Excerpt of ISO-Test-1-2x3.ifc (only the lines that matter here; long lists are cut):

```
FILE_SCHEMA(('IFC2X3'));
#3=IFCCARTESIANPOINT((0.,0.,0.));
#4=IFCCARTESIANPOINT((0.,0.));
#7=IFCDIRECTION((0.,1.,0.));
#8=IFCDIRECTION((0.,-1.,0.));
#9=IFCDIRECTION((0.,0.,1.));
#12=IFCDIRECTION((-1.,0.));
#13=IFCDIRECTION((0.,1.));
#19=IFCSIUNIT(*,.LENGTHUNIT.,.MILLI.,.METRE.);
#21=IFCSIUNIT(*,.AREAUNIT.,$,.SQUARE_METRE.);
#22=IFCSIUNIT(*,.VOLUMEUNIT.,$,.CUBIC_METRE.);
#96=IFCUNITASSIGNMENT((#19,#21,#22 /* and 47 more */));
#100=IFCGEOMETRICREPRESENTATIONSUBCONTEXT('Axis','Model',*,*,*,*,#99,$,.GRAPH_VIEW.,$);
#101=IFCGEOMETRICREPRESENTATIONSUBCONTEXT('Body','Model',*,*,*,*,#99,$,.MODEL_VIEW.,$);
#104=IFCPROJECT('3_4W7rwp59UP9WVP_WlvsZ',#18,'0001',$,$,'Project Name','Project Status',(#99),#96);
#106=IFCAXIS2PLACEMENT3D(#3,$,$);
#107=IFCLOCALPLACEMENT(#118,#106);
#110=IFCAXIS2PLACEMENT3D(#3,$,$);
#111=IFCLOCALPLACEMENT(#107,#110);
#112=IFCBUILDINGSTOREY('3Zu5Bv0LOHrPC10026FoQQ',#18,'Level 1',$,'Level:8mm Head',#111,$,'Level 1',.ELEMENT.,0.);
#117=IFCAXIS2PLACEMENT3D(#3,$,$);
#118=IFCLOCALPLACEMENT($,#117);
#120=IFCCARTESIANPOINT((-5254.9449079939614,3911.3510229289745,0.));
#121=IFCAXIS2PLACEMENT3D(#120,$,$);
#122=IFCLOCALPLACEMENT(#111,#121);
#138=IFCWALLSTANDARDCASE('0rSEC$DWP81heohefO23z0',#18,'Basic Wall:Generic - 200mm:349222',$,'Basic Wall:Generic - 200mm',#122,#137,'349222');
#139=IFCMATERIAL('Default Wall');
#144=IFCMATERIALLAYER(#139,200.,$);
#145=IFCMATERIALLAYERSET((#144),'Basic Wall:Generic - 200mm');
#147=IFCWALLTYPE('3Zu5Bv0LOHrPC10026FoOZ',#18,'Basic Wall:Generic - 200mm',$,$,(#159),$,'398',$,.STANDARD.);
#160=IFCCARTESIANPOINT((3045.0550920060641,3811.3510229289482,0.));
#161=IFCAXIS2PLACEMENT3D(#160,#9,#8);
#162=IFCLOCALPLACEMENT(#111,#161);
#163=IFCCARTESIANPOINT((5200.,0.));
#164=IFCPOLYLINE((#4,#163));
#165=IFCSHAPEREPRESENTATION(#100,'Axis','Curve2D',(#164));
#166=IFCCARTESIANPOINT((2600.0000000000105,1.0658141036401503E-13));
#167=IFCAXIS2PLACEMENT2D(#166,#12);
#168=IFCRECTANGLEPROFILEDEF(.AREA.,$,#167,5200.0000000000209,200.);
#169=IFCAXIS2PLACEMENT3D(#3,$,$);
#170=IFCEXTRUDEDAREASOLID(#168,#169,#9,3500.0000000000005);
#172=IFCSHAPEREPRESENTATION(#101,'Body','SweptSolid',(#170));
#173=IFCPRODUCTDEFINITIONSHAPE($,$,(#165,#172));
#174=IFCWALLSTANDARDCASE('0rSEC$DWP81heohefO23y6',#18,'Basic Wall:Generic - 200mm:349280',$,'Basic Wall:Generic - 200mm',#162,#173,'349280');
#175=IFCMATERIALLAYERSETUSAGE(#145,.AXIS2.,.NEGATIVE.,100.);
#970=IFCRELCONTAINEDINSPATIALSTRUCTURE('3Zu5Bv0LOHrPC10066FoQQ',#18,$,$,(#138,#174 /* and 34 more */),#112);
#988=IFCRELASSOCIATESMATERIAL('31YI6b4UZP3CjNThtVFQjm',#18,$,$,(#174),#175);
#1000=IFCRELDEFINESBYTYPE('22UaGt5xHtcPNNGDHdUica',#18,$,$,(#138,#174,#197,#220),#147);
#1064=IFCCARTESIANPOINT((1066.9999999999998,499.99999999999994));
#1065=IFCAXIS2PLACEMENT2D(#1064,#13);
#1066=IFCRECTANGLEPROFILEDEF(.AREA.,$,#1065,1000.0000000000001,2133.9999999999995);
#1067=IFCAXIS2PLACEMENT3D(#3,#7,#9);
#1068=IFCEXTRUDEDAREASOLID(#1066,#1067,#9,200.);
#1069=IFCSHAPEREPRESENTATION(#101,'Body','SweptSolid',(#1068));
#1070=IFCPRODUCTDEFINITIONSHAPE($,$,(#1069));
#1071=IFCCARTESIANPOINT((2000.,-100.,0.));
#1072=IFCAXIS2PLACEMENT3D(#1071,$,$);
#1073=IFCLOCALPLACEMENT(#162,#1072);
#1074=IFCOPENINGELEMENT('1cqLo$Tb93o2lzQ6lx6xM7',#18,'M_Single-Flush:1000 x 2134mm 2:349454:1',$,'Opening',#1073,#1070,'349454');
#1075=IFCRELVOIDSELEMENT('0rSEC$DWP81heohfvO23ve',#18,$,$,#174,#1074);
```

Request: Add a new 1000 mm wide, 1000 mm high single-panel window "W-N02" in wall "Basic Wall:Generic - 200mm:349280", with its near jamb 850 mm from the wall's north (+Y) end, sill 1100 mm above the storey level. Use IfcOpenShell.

```python
import numpy as np
import ifcopenshell
import ifcopenshell.api.feature
import ifcopenshell.api.geometry
import ifcopenshell.api.root
import ifcopenshell.api.spatial
import ifcopenshell.api.type
import ifcopenshell.geom
import ifcopenshell.util.element
import ifcopenshell.util.placement
import ifcopenshell.util.representation
import ifcopenshell.util.shape
import ifcopenshell.util.unit

model = ifcopenshell.open("ISO-Test-1-2x3.ifc")
unit_scale = ifcopenshell.util.unit.calculate_unit_scale(model)
settings = ifcopenshell.geom.settings()


def volume(element):
    """Net volume in cubic metres, openings subtracted."""
    shape = ifcopenshell.geom.create_shape(settings, element)
    return ifcopenshell.util.shape.get_volume(shape.geometry)


wall = model.by_id(174)
storey = ifcopenshell.util.element.get_container(wall, ifc_class="IfcBuildingStorey")
context = ifcopenshell.util.representation.get_context(model, "Model", "Body", "MODEL_VIEW")
before = volume(wall)

width, height, from_end, sill = 1, 1, 0.85, 1.1  # metres

# The wall runs along its own X axis, and the end named is its -X end.
wall_shape = ifcopenshell.geom.create_shape(settings, wall)
x, y, z = ifcopenshell.util.shape.get_vertices(wall_shape.geometry).T
start = x.min() + from_end
face, thickness = float(y.min()), float(y.max() - y.min())
wall_matrix = ifcopenshell.util.placement.get_local_placement(wall.ObjectPlacement)
level = ifcopenshell.util.placement.get_local_placement(storey.ObjectPlacement)[2, 3]


def in_wall(x, y):
    """Placement at x, y metres in the wall's axes, at sill height."""
    matrix = wall_matrix.copy()
    matrix[:, 3] = wall_matrix @ np.array([x / unit_scale, y / unit_scale, 0.0, 1.0])
    matrix[2, 3] = level + sill / unit_scale
    return matrix


# Opening: a box that overshoots both wall faces by 50 mm.
opening = ifcopenshell.api.root.create_entity(model, ifc_class="IfcOpeningElement")
box = ifcopenshell.api.geometry.add_wall_representation(
    model, context=context, length=width, height=height, thickness=thickness + 0.1
)
ifcopenshell.api.geometry.assign_representation(model, product=opening, representation=box)
ifcopenshell.api.geometry.edit_object_placement(model, product=opening, matrix=in_wall(start, face - 0.05), is_si=False)
ifcopenshell.api.feature.add_feature(model, feature=opening, element=wall)

window = ifcopenshell.api.root.create_entity(model, ifc_class="IfcWindow", name="W-N02")
window.OverallWidth, window.OverallHeight = width / unit_scale, height / unit_scale
body = ifcopenshell.api.geometry.add_window_representation(
    model,
    context=context,
    overall_width=window.OverallWidth,
    overall_height=window.OverallHeight,
    partition_type="SINGLE_PANEL",
)
ifcopenshell.api.geometry.assign_representation(model, product=window, representation=body)
ifcopenshell.api.spatial.assign_container(model, products=[window], relating_structure=storey)
fills = ifcopenshell.api.feature.add_filling(model, opening=opening, element=window)
fills.OwnerHistory = window.OwnerHistory  # required in IFC2X3

# IFC2X3 keeps the operation on the window style.
style = ifcopenshell.api.root.create_entity(model, ifc_class="IfcWindowStyle", name="W-N02")
style.OperationType, style.ConstructionType = "SINGLE_PANEL", "NOTDEFINED"
style.ParameterTakesPrecedence = style.Sizeable = False
ifcopenshell.api.type.assign_type(model, related_objects=[window], relating_type=style)

# Centre the window in the wall's thickness.
ifcopenshell.api.geometry.edit_object_placement(model, product=window, matrix=in_wall(start, face), is_si=False)
window_shape = ifcopenshell.geom.create_shape(settings, window)
depth = ifcopenshell.util.shape.get_vertices(window_shape.geometry)[:, 1]
offset = face + thickness / 2 - (depth.min() + depth.max()) / 2
ifcopenshell.api.geometry.edit_object_placement(model, product=window, matrix=in_wall(start, offset), is_si=False)

after = volume(wall)

print(f"wall volume {before:.3f} -> {after:.3f} m3")

model.write("ISO-Test-1-2x3_edited.ifc")
```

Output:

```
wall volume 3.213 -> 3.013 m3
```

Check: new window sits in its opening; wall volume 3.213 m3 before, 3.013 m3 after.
